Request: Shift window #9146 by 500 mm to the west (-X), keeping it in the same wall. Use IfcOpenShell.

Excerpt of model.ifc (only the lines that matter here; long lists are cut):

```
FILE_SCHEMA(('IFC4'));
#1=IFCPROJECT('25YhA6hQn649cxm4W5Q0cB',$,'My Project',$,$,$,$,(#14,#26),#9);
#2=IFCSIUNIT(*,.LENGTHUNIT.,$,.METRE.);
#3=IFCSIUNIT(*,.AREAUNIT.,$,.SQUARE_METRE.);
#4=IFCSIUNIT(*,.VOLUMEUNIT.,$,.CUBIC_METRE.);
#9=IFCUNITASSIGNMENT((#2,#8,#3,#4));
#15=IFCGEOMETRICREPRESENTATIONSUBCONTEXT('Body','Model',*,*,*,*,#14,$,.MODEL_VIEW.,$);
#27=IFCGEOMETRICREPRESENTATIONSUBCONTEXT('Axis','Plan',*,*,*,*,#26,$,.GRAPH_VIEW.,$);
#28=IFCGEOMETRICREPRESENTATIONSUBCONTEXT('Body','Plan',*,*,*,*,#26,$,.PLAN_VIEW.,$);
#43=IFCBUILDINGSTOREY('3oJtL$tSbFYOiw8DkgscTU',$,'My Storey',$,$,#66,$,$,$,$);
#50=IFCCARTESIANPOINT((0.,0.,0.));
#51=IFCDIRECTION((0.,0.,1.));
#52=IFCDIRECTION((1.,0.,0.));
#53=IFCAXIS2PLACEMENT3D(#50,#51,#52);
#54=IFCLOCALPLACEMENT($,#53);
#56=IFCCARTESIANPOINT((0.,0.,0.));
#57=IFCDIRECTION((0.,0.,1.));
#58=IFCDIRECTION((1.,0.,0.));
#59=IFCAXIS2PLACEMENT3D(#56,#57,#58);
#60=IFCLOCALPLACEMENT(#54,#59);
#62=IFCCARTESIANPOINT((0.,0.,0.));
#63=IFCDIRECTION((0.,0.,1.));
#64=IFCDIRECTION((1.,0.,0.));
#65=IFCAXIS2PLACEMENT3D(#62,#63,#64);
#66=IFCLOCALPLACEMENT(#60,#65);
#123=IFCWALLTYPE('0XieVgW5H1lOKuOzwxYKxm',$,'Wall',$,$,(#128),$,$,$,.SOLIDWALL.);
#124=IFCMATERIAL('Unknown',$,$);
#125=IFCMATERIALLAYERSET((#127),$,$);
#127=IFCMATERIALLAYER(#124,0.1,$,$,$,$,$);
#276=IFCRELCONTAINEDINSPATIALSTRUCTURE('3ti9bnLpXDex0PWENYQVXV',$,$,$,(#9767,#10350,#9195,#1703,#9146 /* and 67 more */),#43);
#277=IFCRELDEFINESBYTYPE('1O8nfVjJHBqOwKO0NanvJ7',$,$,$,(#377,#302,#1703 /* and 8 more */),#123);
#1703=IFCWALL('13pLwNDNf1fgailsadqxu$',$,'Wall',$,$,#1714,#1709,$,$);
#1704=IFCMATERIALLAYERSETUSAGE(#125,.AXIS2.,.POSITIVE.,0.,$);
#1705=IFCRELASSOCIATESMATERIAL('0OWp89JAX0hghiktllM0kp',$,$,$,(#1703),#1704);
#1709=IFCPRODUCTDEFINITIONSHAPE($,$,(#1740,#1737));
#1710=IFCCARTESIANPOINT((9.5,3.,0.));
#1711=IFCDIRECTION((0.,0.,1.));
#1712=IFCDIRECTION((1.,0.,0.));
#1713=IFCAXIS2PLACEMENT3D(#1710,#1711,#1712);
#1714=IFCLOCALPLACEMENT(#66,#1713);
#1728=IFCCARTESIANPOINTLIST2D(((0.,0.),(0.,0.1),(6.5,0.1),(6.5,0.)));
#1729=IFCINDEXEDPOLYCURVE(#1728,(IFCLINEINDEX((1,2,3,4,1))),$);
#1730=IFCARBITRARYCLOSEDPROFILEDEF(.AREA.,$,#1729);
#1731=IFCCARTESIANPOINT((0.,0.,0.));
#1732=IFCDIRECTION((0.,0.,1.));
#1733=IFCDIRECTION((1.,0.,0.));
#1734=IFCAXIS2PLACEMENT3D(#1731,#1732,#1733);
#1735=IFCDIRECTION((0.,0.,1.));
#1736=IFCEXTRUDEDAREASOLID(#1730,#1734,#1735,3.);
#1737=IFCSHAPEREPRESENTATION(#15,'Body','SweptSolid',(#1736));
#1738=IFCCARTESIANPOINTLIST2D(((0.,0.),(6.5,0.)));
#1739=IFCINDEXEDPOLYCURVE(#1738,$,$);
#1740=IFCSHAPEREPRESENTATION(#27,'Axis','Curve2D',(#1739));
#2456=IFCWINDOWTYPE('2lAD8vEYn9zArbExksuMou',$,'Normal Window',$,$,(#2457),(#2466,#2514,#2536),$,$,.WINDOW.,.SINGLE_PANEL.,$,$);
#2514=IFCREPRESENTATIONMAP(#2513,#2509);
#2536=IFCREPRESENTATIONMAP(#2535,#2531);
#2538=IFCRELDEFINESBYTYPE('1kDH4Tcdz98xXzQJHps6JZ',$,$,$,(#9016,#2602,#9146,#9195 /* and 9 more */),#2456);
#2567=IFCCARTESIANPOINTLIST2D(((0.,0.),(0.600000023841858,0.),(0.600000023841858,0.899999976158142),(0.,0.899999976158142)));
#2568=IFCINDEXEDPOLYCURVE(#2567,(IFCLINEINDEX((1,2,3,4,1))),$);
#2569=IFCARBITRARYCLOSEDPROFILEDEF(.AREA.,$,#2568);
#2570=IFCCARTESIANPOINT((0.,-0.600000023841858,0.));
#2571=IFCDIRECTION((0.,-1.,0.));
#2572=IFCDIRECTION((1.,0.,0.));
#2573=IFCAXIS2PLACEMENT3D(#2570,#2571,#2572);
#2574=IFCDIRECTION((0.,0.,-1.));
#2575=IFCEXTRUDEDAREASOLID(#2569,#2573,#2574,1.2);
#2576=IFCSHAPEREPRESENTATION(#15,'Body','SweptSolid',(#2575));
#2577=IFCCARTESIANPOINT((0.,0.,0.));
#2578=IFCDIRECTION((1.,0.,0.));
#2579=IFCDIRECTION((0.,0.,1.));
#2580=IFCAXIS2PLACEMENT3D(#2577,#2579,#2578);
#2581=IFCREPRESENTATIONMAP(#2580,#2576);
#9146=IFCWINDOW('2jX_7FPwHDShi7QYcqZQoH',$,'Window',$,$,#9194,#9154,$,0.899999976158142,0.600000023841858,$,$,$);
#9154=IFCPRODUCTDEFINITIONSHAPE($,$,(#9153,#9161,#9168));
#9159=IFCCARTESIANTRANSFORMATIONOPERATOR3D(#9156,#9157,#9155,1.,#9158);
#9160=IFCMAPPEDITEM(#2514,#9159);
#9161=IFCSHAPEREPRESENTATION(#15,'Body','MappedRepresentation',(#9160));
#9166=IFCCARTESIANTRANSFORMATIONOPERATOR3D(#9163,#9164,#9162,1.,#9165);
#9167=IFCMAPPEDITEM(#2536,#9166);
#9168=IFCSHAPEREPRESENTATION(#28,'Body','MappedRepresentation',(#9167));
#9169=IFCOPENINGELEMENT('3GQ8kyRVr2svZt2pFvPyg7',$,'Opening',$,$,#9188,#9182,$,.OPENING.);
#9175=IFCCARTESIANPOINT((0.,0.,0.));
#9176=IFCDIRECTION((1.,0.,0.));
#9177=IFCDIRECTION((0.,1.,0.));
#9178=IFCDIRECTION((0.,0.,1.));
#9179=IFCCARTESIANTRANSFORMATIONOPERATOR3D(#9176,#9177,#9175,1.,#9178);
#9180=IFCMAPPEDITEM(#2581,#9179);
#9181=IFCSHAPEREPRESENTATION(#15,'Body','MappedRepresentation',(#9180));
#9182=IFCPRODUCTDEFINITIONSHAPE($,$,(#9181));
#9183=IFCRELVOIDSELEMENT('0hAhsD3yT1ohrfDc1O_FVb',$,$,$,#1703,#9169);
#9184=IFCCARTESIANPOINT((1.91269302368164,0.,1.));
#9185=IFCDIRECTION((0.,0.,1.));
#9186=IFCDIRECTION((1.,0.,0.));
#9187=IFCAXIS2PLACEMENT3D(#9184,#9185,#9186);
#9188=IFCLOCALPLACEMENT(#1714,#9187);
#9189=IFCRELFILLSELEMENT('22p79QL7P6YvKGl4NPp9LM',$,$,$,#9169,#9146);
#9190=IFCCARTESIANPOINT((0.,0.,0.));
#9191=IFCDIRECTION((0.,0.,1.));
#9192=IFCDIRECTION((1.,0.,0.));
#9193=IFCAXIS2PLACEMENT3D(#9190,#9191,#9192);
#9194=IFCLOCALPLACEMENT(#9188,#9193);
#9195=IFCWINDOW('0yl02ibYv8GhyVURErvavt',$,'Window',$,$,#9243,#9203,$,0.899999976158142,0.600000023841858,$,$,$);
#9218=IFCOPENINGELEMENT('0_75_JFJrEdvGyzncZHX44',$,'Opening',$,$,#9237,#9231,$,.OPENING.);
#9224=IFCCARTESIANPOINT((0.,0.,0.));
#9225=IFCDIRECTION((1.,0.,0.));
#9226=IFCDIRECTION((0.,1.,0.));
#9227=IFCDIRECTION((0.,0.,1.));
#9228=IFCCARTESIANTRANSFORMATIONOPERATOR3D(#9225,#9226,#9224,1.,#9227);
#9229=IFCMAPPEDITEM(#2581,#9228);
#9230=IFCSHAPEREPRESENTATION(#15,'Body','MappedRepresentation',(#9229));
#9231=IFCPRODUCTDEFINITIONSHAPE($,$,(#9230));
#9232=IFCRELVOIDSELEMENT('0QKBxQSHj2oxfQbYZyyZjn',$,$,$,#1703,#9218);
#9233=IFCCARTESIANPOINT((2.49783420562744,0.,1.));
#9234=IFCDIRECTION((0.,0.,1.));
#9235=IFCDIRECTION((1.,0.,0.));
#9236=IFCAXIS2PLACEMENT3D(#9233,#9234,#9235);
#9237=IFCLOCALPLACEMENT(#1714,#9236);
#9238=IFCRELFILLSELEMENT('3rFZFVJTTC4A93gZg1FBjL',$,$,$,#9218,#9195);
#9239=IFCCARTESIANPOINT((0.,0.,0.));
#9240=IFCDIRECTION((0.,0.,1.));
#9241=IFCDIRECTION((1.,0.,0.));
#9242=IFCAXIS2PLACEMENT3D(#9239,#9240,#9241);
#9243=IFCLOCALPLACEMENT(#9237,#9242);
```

```python
import ifcopenshell
import ifcopenshell.api.geometry
import ifcopenshell.util.placement
import ifcopenshell.util.unit

model = ifcopenshell.open("model.ifc")
unit_scale = ifcopenshell.util.unit.calculate_unit_scale(model)

window = model.by_guid("2jX_7FPwHDShi7QYcqZQoH")
opening = window.FillsVoids[0].RelatingOpeningElement
wall = opening.VoidsElements[0].RelatingBuildingElement

wall_matrix = ifcopenshell.util.placement.get_local_placement(wall.ObjectPlacement)
shift = wall_matrix[:3, 0] * -0.5 / unit_scale
before = ifcopenshell.util.placement.get_local_placement(window.ObjectPlacement)[:3, 3].copy()

# The window is placed relative to its opening, so it follows when the opening moves.
matrix = ifcopenshell.util.placement.get_local_placement(opening.ObjectPlacement)
matrix[:3, 3] += shift
ifcopenshell.api.geometry.edit_object_placement(
    model, product=opening, matrix=matrix, is_si=False, should_transform_children=True
)

after = ifcopenshell.util.placement.get_local_placement(window.ObjectPlacement)[:3, 3]
print("window moved by", (after - before).round(3) + 0.0)

model.write("model_rev.ifc")
```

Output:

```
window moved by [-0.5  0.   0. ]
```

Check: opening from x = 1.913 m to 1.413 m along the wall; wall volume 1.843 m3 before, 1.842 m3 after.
